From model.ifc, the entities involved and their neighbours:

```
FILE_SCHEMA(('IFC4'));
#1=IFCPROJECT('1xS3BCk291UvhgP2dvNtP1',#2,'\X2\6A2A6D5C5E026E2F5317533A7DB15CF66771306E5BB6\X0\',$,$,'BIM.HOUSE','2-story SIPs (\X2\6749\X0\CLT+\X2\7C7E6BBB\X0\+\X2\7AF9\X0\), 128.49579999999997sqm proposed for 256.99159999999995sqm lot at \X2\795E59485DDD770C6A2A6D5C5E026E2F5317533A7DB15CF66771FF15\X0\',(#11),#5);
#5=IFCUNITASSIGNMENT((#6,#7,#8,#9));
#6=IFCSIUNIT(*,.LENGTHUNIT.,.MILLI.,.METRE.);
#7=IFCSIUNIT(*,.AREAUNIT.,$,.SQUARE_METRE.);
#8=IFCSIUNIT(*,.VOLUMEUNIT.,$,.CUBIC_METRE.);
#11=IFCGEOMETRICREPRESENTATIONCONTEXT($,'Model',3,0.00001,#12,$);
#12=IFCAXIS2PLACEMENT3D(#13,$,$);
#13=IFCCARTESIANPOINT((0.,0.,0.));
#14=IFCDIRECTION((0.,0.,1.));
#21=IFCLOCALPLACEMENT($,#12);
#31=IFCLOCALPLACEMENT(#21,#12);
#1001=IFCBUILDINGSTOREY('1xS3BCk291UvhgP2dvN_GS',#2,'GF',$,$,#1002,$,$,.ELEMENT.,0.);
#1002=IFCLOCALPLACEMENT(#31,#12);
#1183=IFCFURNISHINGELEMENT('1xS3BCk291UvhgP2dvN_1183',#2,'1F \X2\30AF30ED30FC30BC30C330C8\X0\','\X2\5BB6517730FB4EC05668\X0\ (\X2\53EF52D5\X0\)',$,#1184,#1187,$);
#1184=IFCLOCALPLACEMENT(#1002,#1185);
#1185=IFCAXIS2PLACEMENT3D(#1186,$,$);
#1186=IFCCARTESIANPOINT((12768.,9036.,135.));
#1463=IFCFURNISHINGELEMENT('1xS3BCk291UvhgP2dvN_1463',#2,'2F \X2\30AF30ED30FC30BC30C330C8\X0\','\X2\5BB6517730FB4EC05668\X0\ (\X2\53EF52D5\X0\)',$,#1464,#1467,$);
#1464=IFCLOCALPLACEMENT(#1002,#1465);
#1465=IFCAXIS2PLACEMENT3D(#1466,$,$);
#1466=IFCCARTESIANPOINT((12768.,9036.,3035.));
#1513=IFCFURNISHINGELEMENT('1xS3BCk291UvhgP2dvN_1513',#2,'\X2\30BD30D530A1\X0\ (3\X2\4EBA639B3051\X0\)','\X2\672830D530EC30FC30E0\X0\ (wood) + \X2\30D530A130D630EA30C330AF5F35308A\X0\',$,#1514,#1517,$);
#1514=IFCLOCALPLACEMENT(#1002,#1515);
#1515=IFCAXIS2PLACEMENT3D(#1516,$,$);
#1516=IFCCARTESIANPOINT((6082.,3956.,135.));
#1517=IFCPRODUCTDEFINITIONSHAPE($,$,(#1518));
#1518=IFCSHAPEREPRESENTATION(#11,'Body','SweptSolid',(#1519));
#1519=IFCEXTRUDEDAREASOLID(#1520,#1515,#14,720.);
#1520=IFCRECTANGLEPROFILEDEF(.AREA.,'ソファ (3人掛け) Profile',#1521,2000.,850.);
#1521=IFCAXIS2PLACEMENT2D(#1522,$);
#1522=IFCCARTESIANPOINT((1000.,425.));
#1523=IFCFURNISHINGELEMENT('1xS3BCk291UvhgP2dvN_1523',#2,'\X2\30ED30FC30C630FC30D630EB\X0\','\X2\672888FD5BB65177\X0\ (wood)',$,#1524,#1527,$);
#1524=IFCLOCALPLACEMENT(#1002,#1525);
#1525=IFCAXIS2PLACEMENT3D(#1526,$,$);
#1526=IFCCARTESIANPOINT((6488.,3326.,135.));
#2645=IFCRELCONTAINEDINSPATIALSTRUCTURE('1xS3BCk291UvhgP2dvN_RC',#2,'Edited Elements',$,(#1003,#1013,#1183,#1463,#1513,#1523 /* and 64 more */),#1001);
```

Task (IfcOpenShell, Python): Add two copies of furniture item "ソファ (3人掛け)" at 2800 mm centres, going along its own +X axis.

```python
import ifcopenshell
import ifcopenshell.api.geometry
import ifcopenshell.api.root
import ifcopenshell.util.element
import ifcopenshell.util.placement

model = ifcopenshell.open("model.ifc")


def reuse_history(source, copy):
    """copy_class also copies each property set's owner history, people and application; keep the originals."""
    for rel in copy.IsDefinedBy:
        if rel.is_a("IfcRelDefinesByProperties") and (history := rel.RelatingPropertyDefinition.OwnerHistory):
            rel.RelatingPropertyDefinition.OwnerHistory = source.OwnerHistory
            ifcopenshell.util.element.remove_deep2(model, history)


source = model.by_id(1513)
base = ifcopenshell.util.placement.get_local_placement(source.ObjectPlacement)
step = base[:3, 0] * 2800.0

for i in range(1, 3):
    copy = ifcopenshell.api.root.copy_class(model, product=source)
    copy.Representation = ifcopenshell.util.element.copy_deep(
        model, source.Representation, exclude=["IfcGeometricRepresentationContext", "IfcRepresentationMap"]
    )
    reuse_history(source, copy)
    matrix = base.copy()
    matrix[:3, 3] += i * step
    print("added at", matrix[:3, 3].round(3) + 0.0)
    ifcopenshell.api.geometry.edit_object_placement(model, product=copy, matrix=matrix, is_si=False)

model.write("model_updated.ifc")
```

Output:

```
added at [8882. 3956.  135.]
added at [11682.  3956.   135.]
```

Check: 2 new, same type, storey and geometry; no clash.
